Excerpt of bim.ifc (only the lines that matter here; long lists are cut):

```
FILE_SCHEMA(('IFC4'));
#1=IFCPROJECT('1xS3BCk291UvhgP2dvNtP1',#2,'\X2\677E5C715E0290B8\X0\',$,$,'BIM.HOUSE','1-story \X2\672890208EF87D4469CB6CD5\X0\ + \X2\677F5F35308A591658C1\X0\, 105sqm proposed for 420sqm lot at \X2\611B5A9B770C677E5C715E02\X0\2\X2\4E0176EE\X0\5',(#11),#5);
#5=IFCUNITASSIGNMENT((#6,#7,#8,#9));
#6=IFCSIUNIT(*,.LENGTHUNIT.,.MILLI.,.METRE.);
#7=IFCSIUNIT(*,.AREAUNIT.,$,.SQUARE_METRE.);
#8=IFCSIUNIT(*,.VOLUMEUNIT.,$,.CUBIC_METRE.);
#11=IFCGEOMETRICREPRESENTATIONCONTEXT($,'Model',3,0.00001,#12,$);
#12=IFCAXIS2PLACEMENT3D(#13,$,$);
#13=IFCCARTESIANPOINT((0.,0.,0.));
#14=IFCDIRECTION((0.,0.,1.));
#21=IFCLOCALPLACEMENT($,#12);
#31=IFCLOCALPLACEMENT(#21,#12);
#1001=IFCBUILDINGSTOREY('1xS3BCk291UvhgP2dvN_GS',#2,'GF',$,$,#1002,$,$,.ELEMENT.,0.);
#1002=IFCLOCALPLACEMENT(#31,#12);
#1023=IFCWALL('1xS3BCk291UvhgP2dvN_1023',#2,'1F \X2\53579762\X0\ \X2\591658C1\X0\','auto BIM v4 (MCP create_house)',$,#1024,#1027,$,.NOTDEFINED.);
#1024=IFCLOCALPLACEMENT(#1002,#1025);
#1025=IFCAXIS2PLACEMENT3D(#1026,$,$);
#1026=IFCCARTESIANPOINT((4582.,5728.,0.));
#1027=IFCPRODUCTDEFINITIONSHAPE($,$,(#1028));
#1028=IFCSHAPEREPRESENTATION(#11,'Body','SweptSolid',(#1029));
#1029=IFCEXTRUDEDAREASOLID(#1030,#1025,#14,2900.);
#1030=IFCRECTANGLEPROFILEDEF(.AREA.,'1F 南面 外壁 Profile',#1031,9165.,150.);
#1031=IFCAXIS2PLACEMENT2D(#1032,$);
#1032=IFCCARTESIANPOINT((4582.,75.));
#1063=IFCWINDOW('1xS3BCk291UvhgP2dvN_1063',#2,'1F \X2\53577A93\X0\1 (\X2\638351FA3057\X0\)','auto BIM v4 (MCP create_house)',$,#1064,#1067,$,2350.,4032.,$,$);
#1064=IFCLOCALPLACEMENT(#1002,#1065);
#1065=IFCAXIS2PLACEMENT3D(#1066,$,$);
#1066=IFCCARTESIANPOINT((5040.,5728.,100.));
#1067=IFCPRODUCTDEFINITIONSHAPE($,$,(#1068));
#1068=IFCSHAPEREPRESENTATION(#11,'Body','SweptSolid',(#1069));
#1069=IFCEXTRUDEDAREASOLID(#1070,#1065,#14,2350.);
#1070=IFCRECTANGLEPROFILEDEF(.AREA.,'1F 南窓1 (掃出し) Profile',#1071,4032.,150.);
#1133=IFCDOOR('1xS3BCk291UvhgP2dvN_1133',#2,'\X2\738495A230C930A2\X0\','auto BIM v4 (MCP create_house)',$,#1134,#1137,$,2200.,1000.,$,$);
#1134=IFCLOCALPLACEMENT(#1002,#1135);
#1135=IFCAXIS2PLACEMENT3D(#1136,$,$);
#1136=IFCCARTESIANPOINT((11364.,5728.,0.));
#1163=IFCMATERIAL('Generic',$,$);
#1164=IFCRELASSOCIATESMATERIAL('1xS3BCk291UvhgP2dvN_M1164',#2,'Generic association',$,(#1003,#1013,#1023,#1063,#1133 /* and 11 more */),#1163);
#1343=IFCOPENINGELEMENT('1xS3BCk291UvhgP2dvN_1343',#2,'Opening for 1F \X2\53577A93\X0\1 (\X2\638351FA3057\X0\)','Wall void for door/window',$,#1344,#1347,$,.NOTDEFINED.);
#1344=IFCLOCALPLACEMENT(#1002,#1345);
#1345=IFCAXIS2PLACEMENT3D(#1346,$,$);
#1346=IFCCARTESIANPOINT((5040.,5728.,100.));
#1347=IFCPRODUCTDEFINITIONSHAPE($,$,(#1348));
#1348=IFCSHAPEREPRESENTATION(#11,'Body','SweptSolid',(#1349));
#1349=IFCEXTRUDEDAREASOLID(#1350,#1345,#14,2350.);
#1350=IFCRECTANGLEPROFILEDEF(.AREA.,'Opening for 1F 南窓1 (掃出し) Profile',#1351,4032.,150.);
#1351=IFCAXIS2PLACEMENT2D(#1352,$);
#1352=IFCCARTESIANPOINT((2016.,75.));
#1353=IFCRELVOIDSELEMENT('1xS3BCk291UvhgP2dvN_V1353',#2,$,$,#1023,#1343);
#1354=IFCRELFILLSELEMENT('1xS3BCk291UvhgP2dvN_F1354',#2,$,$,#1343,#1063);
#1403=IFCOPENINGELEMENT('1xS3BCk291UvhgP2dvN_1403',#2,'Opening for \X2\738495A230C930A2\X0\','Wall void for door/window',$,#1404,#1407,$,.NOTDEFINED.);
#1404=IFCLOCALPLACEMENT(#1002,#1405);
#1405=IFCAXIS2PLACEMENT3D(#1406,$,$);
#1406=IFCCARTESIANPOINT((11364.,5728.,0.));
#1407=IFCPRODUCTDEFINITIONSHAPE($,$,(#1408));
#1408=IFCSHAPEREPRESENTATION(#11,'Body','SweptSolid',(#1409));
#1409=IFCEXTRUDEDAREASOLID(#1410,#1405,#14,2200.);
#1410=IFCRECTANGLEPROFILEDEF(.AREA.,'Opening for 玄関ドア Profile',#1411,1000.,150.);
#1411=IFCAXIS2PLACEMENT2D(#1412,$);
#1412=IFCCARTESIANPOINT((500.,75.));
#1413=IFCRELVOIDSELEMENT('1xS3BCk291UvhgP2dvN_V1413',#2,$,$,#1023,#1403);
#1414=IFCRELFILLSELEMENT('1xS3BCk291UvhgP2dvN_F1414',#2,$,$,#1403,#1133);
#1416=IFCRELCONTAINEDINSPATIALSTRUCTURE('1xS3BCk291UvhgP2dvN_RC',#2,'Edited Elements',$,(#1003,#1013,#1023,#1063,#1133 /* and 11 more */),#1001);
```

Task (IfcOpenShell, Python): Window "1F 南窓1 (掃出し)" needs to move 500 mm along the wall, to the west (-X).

```python
import ifcopenshell
import ifcopenshell.api.geometry
import ifcopenshell.util.placement
import ifcopenshell.util.unit

model = ifcopenshell.open("bim.ifc")
unit_scale = ifcopenshell.util.unit.calculate_unit_scale(model)

window = model.by_id(1063)
opening = window.FillsVoids[0].RelatingOpeningElement
wall = opening.VoidsElements[0].RelatingBuildingElement

wall_matrix = ifcopenshell.util.placement.get_local_placement(wall.ObjectPlacement)
shift = wall_matrix[:3, 0] * -0.5 / unit_scale
before = ifcopenshell.util.placement.get_local_placement(window.ObjectPlacement)[:3, 3].copy()

# The window is not placed relative to its opening, so move both.
for product in (opening, window):
    matrix = ifcopenshell.util.placement.get_local_placement(product.ObjectPlacement)
    matrix[:3, 3] += shift
    ifcopenshell.api.geometry.edit_object_placement(model, product=product, matrix=matrix, is_si=False)

after = ifcopenshell.util.placement.get_local_placement(window.ObjectPlacement)[:3, 3]
print("window moved by", (after - before).round(3) + 0.0)

model.write("bim-out.ifc")
```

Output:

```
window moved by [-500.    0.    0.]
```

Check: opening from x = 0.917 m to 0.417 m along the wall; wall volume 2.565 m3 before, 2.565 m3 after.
